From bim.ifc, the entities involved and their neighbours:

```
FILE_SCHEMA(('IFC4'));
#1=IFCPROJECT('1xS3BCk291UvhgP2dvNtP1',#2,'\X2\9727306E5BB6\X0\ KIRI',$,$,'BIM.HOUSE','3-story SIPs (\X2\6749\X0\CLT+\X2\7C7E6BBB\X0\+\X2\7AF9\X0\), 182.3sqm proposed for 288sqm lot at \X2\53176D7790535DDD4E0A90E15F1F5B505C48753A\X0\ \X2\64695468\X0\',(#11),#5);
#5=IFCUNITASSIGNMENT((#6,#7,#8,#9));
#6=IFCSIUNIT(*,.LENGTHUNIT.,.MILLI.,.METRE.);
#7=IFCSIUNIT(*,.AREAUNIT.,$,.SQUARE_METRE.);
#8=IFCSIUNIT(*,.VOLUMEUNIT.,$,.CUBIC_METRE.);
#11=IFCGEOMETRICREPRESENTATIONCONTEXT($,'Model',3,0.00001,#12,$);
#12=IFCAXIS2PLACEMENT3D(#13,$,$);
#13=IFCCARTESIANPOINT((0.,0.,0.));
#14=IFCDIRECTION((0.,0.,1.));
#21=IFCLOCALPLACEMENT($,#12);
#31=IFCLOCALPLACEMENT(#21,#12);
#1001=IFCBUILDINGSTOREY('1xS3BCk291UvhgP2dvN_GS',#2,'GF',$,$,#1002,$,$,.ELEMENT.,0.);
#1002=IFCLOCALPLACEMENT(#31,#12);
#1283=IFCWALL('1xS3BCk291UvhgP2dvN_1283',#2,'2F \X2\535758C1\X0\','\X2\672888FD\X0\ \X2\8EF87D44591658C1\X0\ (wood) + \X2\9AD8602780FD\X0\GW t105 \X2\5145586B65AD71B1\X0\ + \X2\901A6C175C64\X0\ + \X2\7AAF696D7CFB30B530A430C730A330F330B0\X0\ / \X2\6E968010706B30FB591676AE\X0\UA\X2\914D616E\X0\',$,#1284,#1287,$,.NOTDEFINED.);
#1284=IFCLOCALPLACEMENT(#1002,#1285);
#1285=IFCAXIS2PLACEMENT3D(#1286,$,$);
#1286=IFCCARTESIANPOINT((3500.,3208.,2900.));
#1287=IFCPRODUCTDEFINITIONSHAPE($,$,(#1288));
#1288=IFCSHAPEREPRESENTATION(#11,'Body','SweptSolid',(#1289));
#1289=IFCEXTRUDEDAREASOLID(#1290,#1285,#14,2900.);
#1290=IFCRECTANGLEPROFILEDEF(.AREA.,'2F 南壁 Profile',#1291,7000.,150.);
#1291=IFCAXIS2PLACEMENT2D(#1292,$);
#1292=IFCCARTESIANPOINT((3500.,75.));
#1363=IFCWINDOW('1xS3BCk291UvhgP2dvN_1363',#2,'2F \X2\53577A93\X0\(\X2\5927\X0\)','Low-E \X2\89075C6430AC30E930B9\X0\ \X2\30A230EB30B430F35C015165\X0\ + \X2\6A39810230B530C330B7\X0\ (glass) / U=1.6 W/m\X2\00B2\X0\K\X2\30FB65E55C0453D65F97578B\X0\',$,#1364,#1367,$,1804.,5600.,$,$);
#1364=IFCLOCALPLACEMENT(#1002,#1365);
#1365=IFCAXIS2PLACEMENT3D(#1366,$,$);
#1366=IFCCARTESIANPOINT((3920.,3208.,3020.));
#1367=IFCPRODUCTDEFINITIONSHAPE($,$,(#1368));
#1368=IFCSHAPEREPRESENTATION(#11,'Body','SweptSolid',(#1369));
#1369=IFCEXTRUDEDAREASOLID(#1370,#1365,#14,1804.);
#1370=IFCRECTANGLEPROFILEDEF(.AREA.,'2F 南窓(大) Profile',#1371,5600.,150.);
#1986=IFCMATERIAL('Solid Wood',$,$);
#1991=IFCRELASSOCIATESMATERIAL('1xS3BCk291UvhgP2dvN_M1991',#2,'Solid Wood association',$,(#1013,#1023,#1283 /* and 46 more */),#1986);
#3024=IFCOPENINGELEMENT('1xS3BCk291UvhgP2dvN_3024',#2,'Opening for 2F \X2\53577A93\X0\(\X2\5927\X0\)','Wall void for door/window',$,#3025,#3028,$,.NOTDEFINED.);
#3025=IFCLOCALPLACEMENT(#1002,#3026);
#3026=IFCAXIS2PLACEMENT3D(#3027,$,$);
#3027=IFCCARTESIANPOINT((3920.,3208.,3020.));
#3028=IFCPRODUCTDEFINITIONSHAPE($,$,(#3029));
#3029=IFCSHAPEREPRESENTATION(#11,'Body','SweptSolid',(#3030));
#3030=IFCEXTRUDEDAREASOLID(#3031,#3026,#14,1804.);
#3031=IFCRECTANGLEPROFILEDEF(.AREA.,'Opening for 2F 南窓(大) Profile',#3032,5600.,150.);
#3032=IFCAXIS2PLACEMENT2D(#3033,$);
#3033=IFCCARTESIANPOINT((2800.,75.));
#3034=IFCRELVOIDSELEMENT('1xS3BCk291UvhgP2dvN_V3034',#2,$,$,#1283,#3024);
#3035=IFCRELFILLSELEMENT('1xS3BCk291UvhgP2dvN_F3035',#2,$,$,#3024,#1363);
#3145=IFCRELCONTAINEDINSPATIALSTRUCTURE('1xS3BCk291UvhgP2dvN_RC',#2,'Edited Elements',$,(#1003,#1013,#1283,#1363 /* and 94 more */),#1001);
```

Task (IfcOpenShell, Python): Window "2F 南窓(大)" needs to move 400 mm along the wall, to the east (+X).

```python
import ifcopenshell
import ifcopenshell.api.geometry
import ifcopenshell.util.placement
import ifcopenshell.util.unit

model = ifcopenshell.open("bim.ifc")
unit_scale = ifcopenshell.util.unit.calculate_unit_scale(model)

window = model.by_guid("1xS3BCk291UvhgP2dvN_1363")
opening = window.FillsVoids[0].RelatingOpeningElement
wall = opening.VoidsElements[0].RelatingBuildingElement

wall_matrix = ifcopenshell.util.placement.get_local_placement(wall.ObjectPlacement)
shift = wall_matrix[:3, 0] * 0.4 / unit_scale
before = ifcopenshell.util.placement.get_local_placement(window.ObjectPlacement)[:3, 3].copy()

# The window is not placed relative to its opening, so move both.
for product in (opening, window):
    matrix = ifcopenshell.util.placement.get_local_placement(product.ObjectPlacement)
    matrix[:3, 3] += shift
    ifcopenshell.api.geometry.edit_object_placement(model, product=product, matrix=matrix, is_si=False)

after = ifcopenshell.util.placement.get_local_placement(window.ObjectPlacement)[:3, 3]
print("window moved by", (after - before).round(3) + 0.0)

model.write("bim_v2.ifc")
```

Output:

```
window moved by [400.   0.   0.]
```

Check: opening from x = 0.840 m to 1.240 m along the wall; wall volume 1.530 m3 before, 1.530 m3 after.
